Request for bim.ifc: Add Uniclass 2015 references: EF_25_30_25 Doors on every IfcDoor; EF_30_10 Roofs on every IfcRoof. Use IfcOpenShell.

First a look at what the model holds.

```python
import ifcopenshell

model = ifcopenshell.open("bim.ifc")
print(model.schema)
print("classifications:", [c.Name for c in model.by_type("IfcClassification")])
for ifc_class in ("IfcDoor", "IfcRoof", "IfcStair", "IfcWall", "IfcWindow"):
    print(ifc_class, len(model.by_type(ifc_class)))
```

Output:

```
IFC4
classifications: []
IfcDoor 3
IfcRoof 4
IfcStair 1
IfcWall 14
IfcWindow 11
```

```python
import ifcopenshell
import ifcopenshell.api.classification

model = ifcopenshell.open("bim.ifc")

system = ifcopenshell.api.classification.add_classification(model, classification="Uniclass 2015")

codes = {
    "IfcDoor": ("EF_25_30_25", "Doors"),
    "IfcRoof": ("EF_30_10", "Roofs"),
}
for ifc_class, (code, name) in codes.items():
    products = model.by_type(ifc_class)
    ifcopenshell.api.classification.add_reference(
        model, products=products, classification=system, identification=code, name=name
    )
    print(code, len(products))

model.write("bim_updated.ifc")
```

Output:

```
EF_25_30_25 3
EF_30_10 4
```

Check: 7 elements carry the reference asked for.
